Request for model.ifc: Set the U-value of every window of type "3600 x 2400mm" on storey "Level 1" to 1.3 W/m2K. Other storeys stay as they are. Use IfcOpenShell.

First a look at what the model holds.

```python
import ifcopenshell
import ifcopenshell.util.element

model = ifcopenshell.open("model.ifc")
print(model.schema)
storey = next(s for s in model.by_type("IfcBuildingStorey") if s.Name == "Level 1")
windows = [e for e in ifcopenshell.util.element.get_decomposition(storey) if e.is_a("IfcWindow")]
seen = {}
for e in windows:
    element_type = ifcopenshell.util.element.get_type(e)
    key = (element_type.Name if element_type != e and element_type else None, ifcopenshell.util.element.get_pset(e, "Pset_WindowCommon", "ThermalTransmittance"))
    seen[key] = seen.get(key, 0) + 1
for (name, value), count in sorted(seen.items(), key=str):
    print(count, "x", name, "|", value)
```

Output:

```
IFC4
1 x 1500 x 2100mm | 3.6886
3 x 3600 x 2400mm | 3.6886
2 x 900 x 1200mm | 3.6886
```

```python
import ifcopenshell
import ifcopenshell.api.pset
import ifcopenshell.util.element

model = ifcopenshell.open("model.ifc")

storey = next(s for s in model.by_type("IfcBuildingStorey") if s.Name == "Level 1")
windows = [e for e in ifcopenshell.util.element.get_decomposition(storey) if e.is_a("IfcWindow")]

count = 0
for e in windows:
    element_type = ifcopenshell.util.element.get_type(e)
    if element_type in (None, e) or element_type.Name != "3600 x 2400mm":
        continue
    # add_pset returns the element's existing set when there is one.
    pset = ifcopenshell.api.pset.add_pset(model, product=e, name="Pset_WindowCommon")
    ifcopenshell.api.pset.edit_pset(model, pset=pset, properties={"ThermalTransmittance": 1.3})
    count += 1

print(count, "windows updated")

model.write("model-out.ifc")
```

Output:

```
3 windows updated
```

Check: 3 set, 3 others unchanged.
